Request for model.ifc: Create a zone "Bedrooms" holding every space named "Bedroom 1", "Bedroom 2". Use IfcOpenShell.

First a look at what the model holds.

```python
import ifcopenshell

model = ifcopenshell.open("model.ifc")
print(model.schema)
seen = {}
for space in model.by_type("IfcSpace"):
    seen[space.LongName] = seen.get(space.LongName, 0) + 1
for name, count in sorted(seen.items(), key=str):
    print(count, "x", name)
print("zones:", [z.Name for z in model.by_type("IfcZone")][:20])
```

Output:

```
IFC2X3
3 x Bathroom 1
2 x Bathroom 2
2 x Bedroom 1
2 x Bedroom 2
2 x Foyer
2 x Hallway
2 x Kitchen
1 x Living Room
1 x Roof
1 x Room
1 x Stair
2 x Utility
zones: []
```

```python
import ifcopenshell
import ifcopenshell.api.group
import ifcopenshell.api.root

model = ifcopenshell.open("model.ifc")

names = {"Bedroom 1", "Bedroom 2"}
spaces = [s for s in model.by_type("IfcSpace") if s.LongName in names]

zone = ifcopenshell.api.root.create_entity(model, ifc_class="IfcZone", name="Bedrooms")
ifcopenshell.api.group.assign_group(model, products=spaces, group=zone)
print(len(spaces), "spaces in", zone.Name)

model.write("model-out.ifc")
```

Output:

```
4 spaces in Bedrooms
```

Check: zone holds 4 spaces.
